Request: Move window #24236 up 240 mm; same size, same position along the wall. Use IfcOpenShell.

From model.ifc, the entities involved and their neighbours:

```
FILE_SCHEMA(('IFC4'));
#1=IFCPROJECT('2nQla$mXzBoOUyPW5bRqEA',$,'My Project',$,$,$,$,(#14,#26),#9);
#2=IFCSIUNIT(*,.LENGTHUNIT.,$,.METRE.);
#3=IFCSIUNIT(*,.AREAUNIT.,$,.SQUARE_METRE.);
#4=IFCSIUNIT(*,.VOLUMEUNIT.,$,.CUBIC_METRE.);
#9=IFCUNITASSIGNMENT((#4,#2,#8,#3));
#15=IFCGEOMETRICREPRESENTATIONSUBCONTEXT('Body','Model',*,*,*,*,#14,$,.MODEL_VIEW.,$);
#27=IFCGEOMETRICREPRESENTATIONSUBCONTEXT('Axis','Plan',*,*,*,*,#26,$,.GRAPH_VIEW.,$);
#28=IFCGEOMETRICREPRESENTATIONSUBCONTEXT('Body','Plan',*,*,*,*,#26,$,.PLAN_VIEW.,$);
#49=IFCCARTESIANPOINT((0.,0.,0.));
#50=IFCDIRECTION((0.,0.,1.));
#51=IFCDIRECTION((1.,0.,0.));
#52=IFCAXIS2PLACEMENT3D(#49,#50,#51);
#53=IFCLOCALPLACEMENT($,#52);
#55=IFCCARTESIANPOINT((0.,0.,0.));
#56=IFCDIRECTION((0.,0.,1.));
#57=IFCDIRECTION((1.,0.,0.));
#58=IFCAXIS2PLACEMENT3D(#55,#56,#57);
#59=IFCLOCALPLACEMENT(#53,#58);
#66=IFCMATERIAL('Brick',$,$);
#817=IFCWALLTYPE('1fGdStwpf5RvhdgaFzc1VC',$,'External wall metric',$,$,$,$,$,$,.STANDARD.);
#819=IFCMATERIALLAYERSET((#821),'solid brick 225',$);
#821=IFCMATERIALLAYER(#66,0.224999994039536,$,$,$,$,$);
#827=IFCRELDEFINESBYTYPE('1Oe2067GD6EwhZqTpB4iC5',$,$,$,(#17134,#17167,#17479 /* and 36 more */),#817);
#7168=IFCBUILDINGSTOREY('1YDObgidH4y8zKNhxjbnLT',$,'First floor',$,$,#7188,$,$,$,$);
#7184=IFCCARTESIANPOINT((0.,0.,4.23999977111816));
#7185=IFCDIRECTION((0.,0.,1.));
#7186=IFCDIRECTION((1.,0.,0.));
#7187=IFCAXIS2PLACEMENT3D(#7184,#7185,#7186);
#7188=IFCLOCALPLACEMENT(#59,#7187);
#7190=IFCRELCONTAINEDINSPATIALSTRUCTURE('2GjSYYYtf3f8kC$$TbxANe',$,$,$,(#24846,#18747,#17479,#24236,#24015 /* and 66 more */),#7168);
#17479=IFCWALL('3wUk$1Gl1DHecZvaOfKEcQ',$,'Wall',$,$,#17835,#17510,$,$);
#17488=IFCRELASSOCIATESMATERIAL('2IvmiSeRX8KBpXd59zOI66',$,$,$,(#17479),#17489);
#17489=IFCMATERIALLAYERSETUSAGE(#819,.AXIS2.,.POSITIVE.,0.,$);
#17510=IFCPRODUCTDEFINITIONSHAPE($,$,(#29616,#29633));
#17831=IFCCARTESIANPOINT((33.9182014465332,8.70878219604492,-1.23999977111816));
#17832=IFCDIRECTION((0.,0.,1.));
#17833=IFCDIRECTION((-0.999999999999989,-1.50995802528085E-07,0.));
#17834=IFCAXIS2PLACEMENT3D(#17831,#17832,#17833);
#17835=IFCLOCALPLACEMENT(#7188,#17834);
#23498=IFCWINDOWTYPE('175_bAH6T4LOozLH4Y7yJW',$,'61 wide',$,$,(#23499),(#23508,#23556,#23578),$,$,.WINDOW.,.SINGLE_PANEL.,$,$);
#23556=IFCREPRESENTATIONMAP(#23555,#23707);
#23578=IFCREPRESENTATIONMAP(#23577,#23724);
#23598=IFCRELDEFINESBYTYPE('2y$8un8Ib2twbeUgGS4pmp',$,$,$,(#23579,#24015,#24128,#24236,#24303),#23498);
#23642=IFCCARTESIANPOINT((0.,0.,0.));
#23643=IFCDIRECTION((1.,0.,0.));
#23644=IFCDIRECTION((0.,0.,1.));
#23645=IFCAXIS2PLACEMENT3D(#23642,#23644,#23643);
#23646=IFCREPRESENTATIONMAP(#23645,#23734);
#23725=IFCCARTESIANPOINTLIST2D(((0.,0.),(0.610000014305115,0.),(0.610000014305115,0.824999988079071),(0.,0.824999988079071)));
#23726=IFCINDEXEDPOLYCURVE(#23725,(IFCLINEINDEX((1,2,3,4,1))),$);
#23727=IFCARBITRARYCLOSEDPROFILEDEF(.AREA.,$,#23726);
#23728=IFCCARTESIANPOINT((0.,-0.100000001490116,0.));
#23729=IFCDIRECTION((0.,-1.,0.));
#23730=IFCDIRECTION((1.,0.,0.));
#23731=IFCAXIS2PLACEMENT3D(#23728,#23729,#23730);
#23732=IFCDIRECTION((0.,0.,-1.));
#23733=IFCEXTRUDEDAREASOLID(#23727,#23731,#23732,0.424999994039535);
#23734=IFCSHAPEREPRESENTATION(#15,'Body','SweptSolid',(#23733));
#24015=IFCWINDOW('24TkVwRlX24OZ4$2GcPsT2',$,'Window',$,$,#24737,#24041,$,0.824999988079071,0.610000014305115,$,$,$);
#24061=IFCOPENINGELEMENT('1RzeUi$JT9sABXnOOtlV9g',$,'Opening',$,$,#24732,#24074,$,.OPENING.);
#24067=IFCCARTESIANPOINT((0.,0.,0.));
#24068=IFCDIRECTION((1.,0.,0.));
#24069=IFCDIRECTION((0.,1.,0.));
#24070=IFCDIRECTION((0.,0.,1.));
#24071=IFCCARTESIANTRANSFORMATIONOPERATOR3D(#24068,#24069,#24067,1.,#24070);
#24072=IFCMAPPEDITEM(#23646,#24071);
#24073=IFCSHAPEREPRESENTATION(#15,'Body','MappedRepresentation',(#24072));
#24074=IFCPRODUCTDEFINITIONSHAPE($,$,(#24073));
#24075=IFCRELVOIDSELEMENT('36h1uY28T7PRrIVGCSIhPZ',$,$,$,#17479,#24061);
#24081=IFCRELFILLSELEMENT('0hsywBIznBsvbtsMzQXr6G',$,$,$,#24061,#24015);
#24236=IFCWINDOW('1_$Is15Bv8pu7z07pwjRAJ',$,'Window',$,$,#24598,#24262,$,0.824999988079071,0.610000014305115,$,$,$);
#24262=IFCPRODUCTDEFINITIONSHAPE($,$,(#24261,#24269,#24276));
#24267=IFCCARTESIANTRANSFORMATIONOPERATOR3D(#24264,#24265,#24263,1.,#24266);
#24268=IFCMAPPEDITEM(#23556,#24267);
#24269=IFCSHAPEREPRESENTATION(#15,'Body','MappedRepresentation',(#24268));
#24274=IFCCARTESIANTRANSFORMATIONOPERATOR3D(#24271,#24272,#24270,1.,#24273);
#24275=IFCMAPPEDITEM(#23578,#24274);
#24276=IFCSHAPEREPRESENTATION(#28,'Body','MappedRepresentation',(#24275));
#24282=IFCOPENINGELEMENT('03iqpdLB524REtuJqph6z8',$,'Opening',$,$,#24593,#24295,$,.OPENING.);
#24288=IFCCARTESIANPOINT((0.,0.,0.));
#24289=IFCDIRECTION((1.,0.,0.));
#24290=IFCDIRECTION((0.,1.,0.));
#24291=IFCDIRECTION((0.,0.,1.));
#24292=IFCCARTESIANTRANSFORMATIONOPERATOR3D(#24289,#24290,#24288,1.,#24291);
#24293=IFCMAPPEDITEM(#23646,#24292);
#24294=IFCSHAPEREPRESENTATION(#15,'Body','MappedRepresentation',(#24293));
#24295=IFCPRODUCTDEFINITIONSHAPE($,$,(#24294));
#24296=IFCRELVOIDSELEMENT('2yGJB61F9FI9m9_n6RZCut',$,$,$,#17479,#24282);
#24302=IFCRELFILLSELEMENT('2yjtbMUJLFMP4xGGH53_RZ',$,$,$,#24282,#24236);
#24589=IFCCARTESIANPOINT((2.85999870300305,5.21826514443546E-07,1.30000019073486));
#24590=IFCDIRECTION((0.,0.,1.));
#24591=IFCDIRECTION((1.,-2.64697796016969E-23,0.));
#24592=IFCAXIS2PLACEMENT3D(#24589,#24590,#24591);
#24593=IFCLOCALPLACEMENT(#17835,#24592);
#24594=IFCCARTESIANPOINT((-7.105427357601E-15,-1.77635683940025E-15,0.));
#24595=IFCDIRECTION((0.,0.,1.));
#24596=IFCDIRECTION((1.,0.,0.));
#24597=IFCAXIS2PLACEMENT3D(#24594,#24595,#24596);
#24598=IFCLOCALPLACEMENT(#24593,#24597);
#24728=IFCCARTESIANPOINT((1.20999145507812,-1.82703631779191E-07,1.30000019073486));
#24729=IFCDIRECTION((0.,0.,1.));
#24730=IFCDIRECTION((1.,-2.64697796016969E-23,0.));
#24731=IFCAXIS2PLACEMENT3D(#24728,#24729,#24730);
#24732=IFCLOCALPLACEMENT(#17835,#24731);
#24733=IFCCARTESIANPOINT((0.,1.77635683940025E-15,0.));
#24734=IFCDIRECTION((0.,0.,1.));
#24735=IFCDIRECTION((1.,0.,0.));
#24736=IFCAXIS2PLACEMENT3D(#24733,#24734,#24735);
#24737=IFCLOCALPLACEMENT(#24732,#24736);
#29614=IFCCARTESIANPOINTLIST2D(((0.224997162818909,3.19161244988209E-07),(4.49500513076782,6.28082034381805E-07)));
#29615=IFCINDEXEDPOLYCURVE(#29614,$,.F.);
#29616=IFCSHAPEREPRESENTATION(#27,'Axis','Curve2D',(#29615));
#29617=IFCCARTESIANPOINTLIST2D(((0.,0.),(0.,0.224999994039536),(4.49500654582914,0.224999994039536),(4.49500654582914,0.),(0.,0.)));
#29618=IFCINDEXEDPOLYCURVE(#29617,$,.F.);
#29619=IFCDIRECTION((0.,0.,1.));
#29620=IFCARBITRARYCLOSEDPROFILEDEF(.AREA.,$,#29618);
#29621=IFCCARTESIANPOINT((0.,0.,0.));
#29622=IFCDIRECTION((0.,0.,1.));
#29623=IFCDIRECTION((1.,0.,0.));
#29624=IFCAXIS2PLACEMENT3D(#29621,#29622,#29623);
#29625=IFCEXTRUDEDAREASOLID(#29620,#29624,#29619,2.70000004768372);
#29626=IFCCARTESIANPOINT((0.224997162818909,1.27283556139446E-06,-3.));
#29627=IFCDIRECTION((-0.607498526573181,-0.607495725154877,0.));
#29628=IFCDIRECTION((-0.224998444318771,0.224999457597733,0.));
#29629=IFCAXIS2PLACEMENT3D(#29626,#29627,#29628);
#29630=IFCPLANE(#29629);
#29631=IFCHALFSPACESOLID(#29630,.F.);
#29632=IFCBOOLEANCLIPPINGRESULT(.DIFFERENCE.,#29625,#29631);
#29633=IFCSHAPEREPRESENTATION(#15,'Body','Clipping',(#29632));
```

```python
import numpy as np
import ifcopenshell
import ifcopenshell.api.geometry
import ifcopenshell.util.placement
import ifcopenshell.util.unit

model = ifcopenshell.open("model.ifc")
unit_scale = ifcopenshell.util.unit.calculate_unit_scale(model)

window = model.by_id(24236)
opening = window.FillsVoids[0].RelatingOpeningElement
dz = 0.24

shift = np.array([0.0, 0.0, dz])
# The window is placed relative to its opening, so it follows when the opening moves.
matrix = ifcopenshell.util.placement.get_local_placement(opening.ObjectPlacement)
matrix[:3, 3] += shift
ifcopenshell.api.geometry.edit_object_placement(
    model, product=opening, matrix=matrix, is_si=False, should_transform_children=True
)

print(f"moved by {dz * unit_scale:+.3f} m")

model.write("model_rev.ifc")
```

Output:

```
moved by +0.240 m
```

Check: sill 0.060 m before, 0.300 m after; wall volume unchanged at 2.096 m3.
